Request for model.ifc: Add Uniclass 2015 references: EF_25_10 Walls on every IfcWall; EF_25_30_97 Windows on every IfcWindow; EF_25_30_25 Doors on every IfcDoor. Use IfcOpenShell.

First a look at what the model holds.

```python
import ifcopenshell

model = ifcopenshell.open("model.ifc")
print(model.schema)
print("classifications:", [c.Name for c in model.by_type("IfcClassification")])
for ifc_class in ("IfcDoor", "IfcRoof", "IfcStair", "IfcWall", "IfcWindow"):
    print(ifc_class, len(model.by_type(ifc_class)))
```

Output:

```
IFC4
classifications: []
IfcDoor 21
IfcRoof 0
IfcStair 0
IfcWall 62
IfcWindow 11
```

```python
import ifcopenshell
import ifcopenshell.api.classification

model = ifcopenshell.open("model.ifc")

system = ifcopenshell.api.classification.add_classification(model, classification="Uniclass 2015")

codes = {
    "IfcWall": ("EF_25_10", "Walls"),
    "IfcWindow": ("EF_25_30_97", "Windows"),
    "IfcDoor": ("EF_25_30_25", "Doors"),
}
for ifc_class, (code, name) in codes.items():
    products = model.by_type(ifc_class)
    ifcopenshell.api.classification.add_reference(
        model, products=products, classification=system, identification=code, name=name
    )
    print(code, len(products))

model.write("model_v2.ifc")
```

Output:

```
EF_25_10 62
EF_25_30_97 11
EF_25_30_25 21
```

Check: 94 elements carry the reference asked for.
